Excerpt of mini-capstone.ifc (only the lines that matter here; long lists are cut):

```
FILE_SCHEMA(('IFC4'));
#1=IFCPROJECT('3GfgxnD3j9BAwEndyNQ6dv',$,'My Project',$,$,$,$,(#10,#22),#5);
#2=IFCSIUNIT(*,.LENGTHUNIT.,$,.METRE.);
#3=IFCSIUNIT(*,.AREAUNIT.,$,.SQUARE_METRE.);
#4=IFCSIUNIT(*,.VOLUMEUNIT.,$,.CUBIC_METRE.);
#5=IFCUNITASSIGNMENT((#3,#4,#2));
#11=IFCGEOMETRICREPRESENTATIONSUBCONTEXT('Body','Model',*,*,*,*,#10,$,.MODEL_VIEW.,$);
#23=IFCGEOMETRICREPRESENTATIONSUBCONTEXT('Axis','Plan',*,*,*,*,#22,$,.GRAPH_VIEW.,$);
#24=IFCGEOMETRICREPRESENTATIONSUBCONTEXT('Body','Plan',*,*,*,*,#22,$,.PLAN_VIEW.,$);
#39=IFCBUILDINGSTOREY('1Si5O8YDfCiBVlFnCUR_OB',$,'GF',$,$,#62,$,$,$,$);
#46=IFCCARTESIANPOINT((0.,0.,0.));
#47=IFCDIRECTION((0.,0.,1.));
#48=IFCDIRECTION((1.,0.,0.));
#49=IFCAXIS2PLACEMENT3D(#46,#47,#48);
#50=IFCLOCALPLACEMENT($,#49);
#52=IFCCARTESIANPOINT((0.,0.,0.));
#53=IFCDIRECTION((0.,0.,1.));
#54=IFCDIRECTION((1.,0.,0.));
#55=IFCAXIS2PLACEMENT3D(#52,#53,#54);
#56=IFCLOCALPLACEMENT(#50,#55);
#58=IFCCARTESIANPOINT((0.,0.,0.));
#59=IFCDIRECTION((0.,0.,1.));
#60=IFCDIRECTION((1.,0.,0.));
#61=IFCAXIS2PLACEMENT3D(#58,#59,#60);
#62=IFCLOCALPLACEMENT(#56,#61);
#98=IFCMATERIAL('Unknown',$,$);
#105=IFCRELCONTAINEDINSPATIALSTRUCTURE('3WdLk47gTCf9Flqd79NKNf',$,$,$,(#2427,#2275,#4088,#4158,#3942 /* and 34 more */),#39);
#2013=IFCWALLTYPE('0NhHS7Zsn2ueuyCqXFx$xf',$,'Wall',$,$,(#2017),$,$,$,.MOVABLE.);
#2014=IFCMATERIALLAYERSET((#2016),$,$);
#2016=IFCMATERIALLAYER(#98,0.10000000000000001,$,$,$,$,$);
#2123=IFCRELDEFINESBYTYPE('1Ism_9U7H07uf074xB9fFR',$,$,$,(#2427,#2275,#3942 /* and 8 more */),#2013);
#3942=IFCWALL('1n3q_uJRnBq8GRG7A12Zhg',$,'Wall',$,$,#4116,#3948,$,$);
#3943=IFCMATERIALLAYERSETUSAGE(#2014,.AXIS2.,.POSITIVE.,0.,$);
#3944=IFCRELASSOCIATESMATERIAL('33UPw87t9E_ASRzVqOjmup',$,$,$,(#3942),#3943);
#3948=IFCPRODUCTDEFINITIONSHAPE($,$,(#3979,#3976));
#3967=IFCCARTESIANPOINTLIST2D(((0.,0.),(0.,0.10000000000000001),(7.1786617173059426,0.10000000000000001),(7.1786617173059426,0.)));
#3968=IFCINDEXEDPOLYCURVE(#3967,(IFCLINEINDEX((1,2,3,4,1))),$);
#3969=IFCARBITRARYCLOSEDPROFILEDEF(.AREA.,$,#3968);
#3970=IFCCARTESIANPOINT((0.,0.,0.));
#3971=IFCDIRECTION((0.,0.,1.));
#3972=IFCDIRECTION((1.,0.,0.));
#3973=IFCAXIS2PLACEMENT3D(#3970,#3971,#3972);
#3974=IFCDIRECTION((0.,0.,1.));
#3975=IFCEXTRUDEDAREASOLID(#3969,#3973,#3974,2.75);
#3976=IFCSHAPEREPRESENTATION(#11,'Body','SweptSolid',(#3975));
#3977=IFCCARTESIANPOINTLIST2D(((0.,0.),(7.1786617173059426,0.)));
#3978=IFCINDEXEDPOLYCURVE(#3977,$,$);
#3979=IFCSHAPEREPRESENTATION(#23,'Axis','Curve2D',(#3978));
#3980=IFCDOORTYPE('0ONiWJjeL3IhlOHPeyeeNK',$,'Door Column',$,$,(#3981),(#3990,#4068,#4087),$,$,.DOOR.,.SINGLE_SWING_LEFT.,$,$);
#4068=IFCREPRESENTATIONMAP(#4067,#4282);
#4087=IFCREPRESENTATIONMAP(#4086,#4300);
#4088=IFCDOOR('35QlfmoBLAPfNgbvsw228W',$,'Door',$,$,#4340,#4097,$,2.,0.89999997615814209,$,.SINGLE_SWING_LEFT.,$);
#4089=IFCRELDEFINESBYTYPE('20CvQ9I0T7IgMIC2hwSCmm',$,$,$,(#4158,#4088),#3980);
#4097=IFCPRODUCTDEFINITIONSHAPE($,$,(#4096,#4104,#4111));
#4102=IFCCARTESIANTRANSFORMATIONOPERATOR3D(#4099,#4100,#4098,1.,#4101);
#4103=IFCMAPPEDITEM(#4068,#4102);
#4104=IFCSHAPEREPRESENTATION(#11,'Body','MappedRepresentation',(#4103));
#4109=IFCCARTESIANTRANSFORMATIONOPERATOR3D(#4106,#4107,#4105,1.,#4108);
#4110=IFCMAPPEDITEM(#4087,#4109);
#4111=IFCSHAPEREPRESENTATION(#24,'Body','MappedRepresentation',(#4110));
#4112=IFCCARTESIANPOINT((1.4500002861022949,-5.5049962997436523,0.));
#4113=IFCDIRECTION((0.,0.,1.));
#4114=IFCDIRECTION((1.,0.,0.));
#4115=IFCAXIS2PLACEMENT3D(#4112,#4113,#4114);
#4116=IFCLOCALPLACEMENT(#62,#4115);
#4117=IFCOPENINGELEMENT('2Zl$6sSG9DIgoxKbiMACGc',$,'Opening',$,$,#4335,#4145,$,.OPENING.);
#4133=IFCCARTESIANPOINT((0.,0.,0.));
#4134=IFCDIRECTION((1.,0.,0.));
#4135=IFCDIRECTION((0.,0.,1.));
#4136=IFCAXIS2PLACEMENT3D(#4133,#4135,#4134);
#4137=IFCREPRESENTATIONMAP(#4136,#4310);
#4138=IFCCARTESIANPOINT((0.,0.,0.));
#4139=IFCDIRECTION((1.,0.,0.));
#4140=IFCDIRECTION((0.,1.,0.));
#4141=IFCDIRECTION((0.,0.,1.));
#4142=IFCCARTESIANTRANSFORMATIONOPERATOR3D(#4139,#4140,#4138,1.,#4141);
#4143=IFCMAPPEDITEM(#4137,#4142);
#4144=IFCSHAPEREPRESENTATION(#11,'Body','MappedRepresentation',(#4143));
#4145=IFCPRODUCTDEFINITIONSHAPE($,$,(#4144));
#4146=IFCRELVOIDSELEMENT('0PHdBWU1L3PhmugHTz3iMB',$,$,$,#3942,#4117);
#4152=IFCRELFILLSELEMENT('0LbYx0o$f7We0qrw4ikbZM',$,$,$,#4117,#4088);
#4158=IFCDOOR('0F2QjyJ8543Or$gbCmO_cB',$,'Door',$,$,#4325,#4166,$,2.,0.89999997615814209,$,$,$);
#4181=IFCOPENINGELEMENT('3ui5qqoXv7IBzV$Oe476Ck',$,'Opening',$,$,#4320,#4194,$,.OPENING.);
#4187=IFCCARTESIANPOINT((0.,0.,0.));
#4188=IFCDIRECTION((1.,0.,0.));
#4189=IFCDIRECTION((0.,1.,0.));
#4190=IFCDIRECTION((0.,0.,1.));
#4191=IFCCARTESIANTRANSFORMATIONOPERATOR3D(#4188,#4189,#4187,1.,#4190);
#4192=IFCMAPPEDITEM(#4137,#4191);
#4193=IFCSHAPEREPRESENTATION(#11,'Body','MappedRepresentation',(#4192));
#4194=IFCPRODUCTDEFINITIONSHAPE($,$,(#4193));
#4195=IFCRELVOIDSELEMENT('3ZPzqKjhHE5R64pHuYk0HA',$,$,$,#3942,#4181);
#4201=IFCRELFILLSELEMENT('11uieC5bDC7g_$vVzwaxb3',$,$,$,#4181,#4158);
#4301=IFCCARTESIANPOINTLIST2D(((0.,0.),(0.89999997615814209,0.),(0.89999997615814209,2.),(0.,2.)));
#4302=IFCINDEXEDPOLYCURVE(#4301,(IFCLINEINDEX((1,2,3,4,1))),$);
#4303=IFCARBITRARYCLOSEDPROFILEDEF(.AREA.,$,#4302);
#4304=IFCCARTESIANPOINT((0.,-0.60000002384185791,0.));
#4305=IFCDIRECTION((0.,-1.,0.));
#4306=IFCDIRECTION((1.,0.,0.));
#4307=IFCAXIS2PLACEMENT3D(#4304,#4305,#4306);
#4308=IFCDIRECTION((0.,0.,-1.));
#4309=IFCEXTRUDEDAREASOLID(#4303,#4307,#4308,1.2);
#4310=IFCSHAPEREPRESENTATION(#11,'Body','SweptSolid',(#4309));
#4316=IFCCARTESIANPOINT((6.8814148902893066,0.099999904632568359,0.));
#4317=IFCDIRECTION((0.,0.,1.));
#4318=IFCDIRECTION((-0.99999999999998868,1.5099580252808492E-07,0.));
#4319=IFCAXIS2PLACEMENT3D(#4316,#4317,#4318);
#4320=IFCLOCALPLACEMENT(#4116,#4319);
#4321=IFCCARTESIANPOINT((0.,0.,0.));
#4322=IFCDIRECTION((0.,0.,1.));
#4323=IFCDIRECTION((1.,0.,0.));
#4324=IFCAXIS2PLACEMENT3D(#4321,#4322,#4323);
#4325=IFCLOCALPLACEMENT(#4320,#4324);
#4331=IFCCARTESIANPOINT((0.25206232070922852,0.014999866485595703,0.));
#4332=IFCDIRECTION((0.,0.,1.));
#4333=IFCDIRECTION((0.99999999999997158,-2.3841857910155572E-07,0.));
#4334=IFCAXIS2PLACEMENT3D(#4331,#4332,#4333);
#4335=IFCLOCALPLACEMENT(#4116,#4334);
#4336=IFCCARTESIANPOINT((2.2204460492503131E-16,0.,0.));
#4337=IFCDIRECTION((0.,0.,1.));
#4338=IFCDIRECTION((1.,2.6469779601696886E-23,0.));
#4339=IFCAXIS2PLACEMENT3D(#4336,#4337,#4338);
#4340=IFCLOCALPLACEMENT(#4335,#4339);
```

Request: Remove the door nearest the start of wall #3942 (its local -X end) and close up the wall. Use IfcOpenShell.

```python
import ifcopenshell
import ifcopenshell.api.feature
import ifcopenshell.api.root
import ifcopenshell.geom
import ifcopenshell.util.shape

model = ifcopenshell.open("mini-capstone.ifc")
settings = ifcopenshell.geom.settings()


def volume(element):
    """Net volume in cubic metres, openings subtracted."""
    shape = ifcopenshell.geom.create_shape(settings, element)
    return ifcopenshell.util.shape.get_volume(shape.geometry)


door = model.by_id(4088)
opening = door.FillsVoids[0].RelatingOpeningElement
wall = opening.VoidsElements[0].RelatingBuildingElement
before = volume(wall)

ifcopenshell.api.root.remove_product(model, product=door)
ifcopenshell.api.feature.remove_feature(model, feature=opening)

after = volume(wall)

print(f"wall volume {before:.3f} -> {after:.3f} m3")

model.write("mini-capstone_edited.ifc")
```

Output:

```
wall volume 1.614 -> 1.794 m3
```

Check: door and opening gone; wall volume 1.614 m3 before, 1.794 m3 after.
